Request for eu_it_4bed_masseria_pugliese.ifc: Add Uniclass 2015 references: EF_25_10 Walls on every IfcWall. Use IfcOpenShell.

First a look at what the model holds.

```python
import ifcopenshell

model = ifcopenshell.open("eu_it_4bed_masseria_pugliese.ifc")
print(model.schema)
print("classifications:", [c.Name for c in model.by_type("IfcClassification")])
for ifc_class in ("IfcDoor", "IfcRoof", "IfcStair", "IfcWall", "IfcWindow"):
    print(ifc_class, len(model.by_type(ifc_class)))
```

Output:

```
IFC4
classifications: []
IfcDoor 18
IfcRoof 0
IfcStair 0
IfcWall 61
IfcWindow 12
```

```python
import ifcopenshell
import ifcopenshell.api.classification

model = ifcopenshell.open("eu_it_4bed_masseria_pugliese.ifc")

system = ifcopenshell.api.classification.add_classification(model, classification="Uniclass 2015")

codes = {
    "IfcWall": ("EF_25_10", "Walls"),
}
for ifc_class, (code, name) in codes.items():
    products = model.by_type(ifc_class)
    ifcopenshell.api.classification.add_reference(
        model, products=products, classification=system, identification=code, name=name
    )
    print(code, len(products))

model.write("eu_it_4bed_masseria_pugliese-out.ifc")
```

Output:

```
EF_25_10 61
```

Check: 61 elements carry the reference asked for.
